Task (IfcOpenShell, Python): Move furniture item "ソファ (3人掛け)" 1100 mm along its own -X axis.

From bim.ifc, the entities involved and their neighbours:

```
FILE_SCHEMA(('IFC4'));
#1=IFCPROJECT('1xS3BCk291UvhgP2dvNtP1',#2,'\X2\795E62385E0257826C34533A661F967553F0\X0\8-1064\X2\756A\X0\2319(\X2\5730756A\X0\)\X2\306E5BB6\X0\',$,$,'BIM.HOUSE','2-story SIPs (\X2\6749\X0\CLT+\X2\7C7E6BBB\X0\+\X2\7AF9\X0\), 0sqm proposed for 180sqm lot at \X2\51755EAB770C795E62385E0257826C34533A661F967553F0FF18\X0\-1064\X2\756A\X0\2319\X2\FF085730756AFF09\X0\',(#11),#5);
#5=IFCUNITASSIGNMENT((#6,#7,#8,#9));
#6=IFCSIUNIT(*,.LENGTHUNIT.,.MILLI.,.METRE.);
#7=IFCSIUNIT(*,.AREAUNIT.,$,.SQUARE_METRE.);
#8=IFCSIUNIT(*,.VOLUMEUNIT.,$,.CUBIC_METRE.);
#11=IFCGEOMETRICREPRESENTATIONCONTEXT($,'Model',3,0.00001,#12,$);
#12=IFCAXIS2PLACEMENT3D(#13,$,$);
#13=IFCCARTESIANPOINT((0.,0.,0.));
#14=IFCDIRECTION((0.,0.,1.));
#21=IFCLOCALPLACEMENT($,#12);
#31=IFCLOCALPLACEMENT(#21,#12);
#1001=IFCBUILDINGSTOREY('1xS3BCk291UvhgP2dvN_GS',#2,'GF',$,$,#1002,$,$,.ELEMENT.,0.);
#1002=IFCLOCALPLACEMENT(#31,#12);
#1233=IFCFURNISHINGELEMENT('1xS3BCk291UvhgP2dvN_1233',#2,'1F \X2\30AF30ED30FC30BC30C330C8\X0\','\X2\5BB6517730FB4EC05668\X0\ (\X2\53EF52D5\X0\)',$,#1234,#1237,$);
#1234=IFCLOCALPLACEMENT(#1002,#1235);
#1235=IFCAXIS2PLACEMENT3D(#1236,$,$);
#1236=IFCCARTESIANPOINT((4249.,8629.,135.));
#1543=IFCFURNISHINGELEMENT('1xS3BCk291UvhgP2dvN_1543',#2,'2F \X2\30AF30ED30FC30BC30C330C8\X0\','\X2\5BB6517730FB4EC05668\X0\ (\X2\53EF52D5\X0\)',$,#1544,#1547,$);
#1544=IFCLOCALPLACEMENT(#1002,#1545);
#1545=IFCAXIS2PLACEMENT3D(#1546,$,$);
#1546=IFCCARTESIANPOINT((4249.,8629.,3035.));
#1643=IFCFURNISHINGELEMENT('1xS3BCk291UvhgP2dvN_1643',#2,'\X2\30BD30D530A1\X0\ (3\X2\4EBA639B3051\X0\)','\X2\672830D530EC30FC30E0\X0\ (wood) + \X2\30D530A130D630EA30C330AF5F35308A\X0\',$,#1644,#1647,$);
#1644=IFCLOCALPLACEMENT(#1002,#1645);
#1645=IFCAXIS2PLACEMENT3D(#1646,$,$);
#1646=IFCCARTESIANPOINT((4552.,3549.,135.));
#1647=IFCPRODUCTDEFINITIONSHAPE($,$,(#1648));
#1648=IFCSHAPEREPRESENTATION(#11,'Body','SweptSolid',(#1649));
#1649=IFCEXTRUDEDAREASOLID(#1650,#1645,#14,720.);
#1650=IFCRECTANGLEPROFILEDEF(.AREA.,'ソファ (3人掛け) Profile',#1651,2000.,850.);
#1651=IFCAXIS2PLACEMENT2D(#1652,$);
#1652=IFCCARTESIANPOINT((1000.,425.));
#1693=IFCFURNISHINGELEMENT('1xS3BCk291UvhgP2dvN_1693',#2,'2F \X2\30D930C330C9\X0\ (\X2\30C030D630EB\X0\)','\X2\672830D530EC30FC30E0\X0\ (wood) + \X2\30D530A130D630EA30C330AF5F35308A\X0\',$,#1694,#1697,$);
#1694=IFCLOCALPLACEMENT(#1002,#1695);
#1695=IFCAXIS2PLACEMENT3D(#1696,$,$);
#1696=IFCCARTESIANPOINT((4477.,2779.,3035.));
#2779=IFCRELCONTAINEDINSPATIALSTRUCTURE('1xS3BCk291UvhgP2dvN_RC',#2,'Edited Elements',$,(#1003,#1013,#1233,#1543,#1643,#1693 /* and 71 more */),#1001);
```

```python
import ifcopenshell
import ifcopenshell.api.geometry
import ifcopenshell.util.placement
import ifcopenshell.util.unit

model = ifcopenshell.open("bim.ifc")
unit_scale = ifcopenshell.util.unit.calculate_unit_scale(model)

item = model.by_guid("1xS3BCk291UvhgP2dvN_1643")
matrix = ifcopenshell.util.placement.get_local_placement(item.ObjectPlacement)
matrix[:3, 3] -= matrix[:3, 0] * 1.1 / unit_scale
ifcopenshell.api.geometry.edit_object_placement(model, product=item, matrix=matrix, is_si=False)

print(ifcopenshell.util.placement.get_local_placement(item.ObjectPlacement).round(3) + 0.0)

model.write("bim-out.ifc")
```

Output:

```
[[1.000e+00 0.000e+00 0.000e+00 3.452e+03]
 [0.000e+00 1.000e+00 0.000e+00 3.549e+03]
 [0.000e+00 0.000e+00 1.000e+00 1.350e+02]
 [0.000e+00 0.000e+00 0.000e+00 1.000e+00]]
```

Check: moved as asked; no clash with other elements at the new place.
